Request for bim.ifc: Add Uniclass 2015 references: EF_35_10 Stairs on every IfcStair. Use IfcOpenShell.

First a look at what the model holds.

```python
import ifcopenshell

model = ifcopenshell.open("bim.ifc")
print(model.schema)
print("classifications:", [c.Name for c in model.by_type("IfcClassification")])
for ifc_class in ("IfcDoor", "IfcRoof", "IfcStair", "IfcWall", "IfcWindow"):
    print(ifc_class, len(model.by_type(ifc_class)))
```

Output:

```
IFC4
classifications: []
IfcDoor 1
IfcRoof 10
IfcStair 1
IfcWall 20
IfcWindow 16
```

```python
import ifcopenshell
import ifcopenshell.api.classification

model = ifcopenshell.open("bim.ifc")

system = ifcopenshell.api.classification.add_classification(model, classification="Uniclass 2015")

codes = {
    "IfcStair": ("EF_35_10", "Stairs"),
}
for ifc_class, (code, name) in codes.items():
    products = model.by_type(ifc_class)
    ifcopenshell.api.classification.add_reference(
        model, products=products, classification=system, identification=code, name=name
    )
    print(code, len(products))

model.write("bim_updated.ifc")
```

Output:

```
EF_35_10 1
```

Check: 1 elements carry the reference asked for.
